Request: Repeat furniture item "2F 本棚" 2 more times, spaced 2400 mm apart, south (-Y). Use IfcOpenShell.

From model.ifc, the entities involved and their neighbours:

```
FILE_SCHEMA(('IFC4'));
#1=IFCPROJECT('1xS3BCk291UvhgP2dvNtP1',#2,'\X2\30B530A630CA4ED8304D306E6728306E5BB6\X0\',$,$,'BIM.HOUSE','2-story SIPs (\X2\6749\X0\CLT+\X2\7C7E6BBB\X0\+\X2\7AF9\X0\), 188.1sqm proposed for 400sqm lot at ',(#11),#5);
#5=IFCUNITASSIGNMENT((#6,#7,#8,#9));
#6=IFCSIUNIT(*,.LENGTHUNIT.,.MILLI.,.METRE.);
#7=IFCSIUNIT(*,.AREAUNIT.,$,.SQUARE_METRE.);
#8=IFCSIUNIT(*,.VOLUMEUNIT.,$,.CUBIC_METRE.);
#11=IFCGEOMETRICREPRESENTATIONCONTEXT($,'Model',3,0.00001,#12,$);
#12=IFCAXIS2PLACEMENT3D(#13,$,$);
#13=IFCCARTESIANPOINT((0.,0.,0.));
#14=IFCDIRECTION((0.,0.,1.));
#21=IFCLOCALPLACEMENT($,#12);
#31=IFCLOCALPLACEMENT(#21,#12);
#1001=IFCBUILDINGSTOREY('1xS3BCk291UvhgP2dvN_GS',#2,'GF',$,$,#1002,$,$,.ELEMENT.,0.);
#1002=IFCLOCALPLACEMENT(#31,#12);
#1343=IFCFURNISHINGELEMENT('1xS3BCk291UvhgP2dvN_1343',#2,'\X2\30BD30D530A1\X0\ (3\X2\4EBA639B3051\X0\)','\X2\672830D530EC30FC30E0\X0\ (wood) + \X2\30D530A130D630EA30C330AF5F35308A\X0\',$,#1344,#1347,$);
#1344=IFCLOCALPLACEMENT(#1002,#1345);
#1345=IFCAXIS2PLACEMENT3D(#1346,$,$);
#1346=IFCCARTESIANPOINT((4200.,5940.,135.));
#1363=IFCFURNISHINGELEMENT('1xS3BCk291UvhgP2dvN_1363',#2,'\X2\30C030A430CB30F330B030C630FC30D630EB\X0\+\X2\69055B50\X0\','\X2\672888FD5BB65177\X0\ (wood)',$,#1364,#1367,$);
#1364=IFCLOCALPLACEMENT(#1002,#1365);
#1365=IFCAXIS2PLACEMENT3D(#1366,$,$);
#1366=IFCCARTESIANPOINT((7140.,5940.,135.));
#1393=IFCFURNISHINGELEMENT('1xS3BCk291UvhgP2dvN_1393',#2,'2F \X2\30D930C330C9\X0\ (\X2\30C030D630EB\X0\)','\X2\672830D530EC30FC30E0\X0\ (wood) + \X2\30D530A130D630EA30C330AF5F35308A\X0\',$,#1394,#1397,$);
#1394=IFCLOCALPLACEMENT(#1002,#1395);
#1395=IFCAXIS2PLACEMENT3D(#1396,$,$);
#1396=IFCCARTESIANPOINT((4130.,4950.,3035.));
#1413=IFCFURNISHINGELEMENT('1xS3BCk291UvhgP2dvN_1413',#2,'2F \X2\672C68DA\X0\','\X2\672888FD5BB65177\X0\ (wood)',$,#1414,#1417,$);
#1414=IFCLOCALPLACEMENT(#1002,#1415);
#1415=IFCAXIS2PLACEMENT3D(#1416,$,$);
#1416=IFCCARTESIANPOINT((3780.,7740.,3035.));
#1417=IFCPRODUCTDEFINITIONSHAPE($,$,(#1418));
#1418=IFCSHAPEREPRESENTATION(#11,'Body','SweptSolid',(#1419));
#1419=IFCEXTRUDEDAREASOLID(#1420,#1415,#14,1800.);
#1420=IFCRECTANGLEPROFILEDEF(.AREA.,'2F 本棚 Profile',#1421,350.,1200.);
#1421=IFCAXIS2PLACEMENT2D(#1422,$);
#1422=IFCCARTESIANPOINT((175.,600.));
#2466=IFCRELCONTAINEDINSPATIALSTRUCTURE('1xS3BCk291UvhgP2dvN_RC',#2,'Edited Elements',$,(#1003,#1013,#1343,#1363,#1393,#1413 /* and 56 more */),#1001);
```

```python
import numpy as np
import ifcopenshell
import ifcopenshell.api.geometry
import ifcopenshell.api.root
import ifcopenshell.util.element
import ifcopenshell.util.placement

model = ifcopenshell.open("model.ifc")


def reuse_history(source, copy):
    """copy_class also copies each property set's owner history, people and application; keep the originals."""
    for rel in copy.IsDefinedBy:
        if rel.is_a("IfcRelDefinesByProperties") and (history := rel.RelatingPropertyDefinition.OwnerHistory):
            rel.RelatingPropertyDefinition.OwnerHistory = source.OwnerHistory
            ifcopenshell.util.element.remove_deep2(model, history)


source = model.by_id(1413)
base = ifcopenshell.util.placement.get_local_placement(source.ObjectPlacement)
step = np.array([0.0, -1.0, 0.0]) * 2400.0

for i in range(1, 3):
    copy = ifcopenshell.api.root.copy_class(model, product=source)
    copy.Representation = ifcopenshell.util.element.copy_deep(
        model, source.Representation, exclude=["IfcGeometricRepresentationContext", "IfcRepresentationMap"]
    )
    reuse_history(source, copy)
    matrix = base.copy()
    matrix[:3, 3] += i * step
    print("added at", matrix[:3, 3].round(3) + 0.0)
    ifcopenshell.api.geometry.edit_object_placement(model, product=copy, matrix=matrix, is_si=False)

model.write("model_edited.ifc")
```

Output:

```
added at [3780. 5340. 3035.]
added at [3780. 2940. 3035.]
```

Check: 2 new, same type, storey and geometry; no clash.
